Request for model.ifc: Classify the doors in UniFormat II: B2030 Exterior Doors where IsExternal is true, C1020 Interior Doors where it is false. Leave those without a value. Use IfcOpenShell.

First a look at what the model holds.

```python
import ifcopenshell
import ifcopenshell.util.element

model = ifcopenshell.open("model.ifc")
print(model.schema)
print("classifications:", [c.Name for c in model.by_type("IfcClassification")])
values = [ifcopenshell.util.element.get_pset(e, "Pset_DoorCommon", "IsExternal") for e in model.by_type("IfcDoor")]
for value in (True, False, None):
    print("IsExternal", value, values.count(value))
```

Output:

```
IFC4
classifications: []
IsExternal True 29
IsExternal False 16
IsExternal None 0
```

```python
import ifcopenshell
import ifcopenshell.api.classification
import ifcopenshell.util.element

model = ifcopenshell.open("model.ifc")

system = ifcopenshell.api.classification.add_classification(model, classification="UniFormat II")

doors = model.by_type("IfcDoor")
external = {e: ifcopenshell.util.element.get_pset(e, "Pset_DoorCommon", "IsExternal") for e in doors}
for flag, code, name in ((True, "B2030", "Exterior Doors"), (False, "C1020", "Interior Doors")):
    products = [e for e in doors if external[e] is flag]
    ifcopenshell.api.classification.add_reference(
        model, products=products, classification=system, identification=code, name=name
    )
    print(code, len(products))

model.write("model-out.ifc")
```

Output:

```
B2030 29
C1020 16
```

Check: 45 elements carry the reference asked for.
